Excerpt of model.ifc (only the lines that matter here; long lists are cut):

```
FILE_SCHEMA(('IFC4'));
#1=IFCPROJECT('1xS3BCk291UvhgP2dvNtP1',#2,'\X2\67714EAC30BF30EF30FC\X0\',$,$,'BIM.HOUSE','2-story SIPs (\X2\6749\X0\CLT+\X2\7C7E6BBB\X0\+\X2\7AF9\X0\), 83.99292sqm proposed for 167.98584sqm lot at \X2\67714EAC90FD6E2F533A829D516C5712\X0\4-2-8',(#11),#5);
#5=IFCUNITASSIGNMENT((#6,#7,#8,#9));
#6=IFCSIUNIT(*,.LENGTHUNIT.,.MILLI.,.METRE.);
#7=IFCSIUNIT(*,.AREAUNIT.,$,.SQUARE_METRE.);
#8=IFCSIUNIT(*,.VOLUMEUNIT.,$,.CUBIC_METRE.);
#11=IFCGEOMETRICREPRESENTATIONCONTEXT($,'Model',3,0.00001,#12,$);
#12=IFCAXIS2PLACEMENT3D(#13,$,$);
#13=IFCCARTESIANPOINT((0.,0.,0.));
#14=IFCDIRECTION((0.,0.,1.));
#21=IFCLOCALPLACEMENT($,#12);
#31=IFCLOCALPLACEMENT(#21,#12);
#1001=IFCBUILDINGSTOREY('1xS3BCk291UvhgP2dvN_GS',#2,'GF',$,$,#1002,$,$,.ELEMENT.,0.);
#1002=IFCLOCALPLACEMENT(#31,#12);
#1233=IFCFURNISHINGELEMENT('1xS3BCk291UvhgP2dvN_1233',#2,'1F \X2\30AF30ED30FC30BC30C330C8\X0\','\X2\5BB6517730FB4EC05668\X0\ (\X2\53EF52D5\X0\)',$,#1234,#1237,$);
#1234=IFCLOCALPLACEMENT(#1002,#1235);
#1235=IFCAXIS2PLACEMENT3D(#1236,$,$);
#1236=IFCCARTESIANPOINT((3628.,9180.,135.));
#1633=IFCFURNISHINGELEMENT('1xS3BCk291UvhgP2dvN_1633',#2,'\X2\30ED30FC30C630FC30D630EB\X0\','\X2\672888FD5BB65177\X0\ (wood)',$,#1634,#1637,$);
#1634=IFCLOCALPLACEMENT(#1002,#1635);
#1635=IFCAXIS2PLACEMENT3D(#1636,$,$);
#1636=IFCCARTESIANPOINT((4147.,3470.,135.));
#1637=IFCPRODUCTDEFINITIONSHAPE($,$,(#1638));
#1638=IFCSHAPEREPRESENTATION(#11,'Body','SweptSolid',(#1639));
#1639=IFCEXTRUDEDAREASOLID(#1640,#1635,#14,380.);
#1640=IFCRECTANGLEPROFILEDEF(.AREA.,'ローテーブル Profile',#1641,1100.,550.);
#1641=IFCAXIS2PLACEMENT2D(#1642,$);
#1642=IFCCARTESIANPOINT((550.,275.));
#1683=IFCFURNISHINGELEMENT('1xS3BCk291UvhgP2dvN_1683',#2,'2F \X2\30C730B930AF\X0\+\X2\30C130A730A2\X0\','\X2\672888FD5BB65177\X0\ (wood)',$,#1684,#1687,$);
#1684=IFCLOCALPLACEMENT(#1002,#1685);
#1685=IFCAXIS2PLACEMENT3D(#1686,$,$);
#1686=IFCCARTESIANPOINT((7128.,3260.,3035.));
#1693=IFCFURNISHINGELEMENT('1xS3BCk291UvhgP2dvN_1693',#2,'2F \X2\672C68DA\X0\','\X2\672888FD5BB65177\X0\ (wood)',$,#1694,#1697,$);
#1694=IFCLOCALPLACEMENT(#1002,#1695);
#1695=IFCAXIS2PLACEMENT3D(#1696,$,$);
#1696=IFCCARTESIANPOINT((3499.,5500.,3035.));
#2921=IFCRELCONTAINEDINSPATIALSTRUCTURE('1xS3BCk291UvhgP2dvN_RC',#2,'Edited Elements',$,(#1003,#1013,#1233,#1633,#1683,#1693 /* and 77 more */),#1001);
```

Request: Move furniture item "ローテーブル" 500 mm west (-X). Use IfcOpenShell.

```python
import ifcopenshell
import ifcopenshell.api.geometry
import ifcopenshell.util.placement

model = ifcopenshell.open("model.ifc")

item = model.by_guid("1xS3BCk291UvhgP2dvN_1633")
matrix = ifcopenshell.util.placement.get_local_placement(item.ObjectPlacement)
matrix[0, 3] -= 500.0
ifcopenshell.api.geometry.edit_object_placement(model, product=item, matrix=matrix, is_si=False)

print(ifcopenshell.util.placement.get_local_placement(item.ObjectPlacement).round(3) + 0.0)

model.write("model-out.ifc")
```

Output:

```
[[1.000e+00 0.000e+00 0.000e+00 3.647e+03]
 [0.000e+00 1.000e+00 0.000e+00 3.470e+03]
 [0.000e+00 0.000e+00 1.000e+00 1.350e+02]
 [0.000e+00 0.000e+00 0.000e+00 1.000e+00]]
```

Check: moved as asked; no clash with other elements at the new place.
